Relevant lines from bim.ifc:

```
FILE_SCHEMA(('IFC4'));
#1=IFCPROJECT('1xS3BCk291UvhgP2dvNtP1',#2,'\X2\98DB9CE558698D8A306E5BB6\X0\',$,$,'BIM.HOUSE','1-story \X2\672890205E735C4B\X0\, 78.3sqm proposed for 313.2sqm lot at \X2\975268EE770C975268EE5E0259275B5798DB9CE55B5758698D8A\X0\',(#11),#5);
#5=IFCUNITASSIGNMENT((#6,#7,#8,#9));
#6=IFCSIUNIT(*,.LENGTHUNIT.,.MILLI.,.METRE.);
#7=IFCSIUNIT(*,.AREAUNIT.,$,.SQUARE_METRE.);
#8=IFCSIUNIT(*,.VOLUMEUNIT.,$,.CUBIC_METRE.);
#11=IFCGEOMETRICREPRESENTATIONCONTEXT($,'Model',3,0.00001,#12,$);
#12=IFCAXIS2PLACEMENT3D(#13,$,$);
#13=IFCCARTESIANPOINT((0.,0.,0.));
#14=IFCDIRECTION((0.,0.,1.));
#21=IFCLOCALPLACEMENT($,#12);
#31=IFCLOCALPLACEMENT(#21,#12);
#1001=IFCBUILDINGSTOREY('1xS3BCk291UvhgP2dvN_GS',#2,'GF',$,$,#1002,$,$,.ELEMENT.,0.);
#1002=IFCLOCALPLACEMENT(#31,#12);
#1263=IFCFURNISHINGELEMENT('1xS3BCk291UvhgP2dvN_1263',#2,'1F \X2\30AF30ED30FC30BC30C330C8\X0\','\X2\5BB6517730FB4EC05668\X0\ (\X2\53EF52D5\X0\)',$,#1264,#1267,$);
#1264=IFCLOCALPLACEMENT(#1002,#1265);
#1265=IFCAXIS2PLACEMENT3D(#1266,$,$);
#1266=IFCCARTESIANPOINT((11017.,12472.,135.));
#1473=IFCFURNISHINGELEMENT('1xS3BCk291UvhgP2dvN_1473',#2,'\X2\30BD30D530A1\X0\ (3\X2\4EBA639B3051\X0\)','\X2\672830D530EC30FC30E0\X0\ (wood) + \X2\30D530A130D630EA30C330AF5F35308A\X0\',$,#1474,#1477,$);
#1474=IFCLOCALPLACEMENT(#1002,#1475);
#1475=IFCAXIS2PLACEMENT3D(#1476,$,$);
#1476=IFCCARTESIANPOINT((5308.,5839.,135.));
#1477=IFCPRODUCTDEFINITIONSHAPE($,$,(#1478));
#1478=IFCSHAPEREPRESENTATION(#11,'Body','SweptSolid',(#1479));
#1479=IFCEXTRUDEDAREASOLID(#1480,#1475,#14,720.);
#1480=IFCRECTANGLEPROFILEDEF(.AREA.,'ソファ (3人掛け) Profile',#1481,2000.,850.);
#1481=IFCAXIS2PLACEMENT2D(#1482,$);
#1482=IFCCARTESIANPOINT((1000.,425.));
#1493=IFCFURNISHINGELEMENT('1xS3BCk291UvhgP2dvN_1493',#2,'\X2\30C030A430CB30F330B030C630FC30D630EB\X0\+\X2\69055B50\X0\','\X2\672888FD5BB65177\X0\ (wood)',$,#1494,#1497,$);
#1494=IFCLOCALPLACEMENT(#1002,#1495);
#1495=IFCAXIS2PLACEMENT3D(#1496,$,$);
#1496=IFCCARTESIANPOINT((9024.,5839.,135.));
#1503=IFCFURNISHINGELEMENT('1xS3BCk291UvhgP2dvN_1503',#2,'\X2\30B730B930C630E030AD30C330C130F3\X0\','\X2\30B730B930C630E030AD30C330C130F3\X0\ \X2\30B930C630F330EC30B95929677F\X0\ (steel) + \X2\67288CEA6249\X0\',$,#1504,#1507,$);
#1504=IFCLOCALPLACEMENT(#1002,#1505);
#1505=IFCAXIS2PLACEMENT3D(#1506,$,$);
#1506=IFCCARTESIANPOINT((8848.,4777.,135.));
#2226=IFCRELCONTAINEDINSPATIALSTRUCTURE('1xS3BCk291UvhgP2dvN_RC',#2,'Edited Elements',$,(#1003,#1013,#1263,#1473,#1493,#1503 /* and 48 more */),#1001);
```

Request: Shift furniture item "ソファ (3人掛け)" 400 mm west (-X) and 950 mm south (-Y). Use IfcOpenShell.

```python
import ifcopenshell
import ifcopenshell.api.geometry
import ifcopenshell.util.placement
import ifcopenshell.util.unit

model = ifcopenshell.open("bim.ifc")
unit_scale = ifcopenshell.util.unit.calculate_unit_scale(model)

item = model.by_id(1473)
matrix = ifcopenshell.util.placement.get_local_placement(item.ObjectPlacement)
matrix[0, 3] -= 0.4 / unit_scale
matrix[1, 3] -= 0.95 / unit_scale
ifcopenshell.api.geometry.edit_object_placement(model, product=item, matrix=matrix, is_si=False)

print(ifcopenshell.util.placement.get_local_placement(item.ObjectPlacement).round(3) + 0.0)

model.write("bim_updated.ifc")
```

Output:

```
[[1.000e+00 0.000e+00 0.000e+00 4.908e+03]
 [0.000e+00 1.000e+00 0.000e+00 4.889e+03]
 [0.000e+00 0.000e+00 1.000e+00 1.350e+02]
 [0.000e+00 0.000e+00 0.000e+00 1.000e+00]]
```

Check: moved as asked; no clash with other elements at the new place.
